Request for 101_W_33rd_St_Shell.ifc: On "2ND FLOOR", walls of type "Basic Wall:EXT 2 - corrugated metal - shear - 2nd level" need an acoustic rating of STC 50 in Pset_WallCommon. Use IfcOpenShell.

First a look at what the model holds.

```python
import ifcopenshell
import ifcopenshell.util.element

model = ifcopenshell.open("101_W_33rd_St_Shell.ifc")
print(model.schema)
storey = next(s for s in model.by_type("IfcBuildingStorey") if s.Name == "2ND FLOOR")
walls = [e for e in ifcopenshell.util.element.get_decomposition(storey) if e.is_a("IfcWall")]
seen = {}
for e in walls:
    element_type = ifcopenshell.util.element.get_type(e)
    key = (element_type.Name if element_type != e and element_type else None, ifcopenshell.util.element.get_pset(e, "Pset_WallCommon", "AcousticRating"))
    seen[key] = seen.get(key, 0) + 1
for (name, value), count in sorted(seen.items(), key=str):
    print(count, "x", name, "|", value)
```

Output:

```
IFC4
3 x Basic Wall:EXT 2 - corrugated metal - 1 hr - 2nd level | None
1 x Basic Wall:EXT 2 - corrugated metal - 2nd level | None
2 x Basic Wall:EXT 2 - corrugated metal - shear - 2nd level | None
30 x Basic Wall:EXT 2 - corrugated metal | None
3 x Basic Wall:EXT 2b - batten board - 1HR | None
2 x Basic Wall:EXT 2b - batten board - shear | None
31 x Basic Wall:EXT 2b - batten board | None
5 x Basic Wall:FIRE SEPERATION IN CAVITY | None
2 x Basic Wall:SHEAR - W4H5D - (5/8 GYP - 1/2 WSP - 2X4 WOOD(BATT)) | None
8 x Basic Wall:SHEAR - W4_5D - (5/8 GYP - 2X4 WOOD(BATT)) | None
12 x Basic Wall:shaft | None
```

```python
import ifcopenshell
import ifcopenshell.api.pset
import ifcopenshell.util.element

model = ifcopenshell.open("101_W_33rd_St_Shell.ifc")

storey = next(s for s in model.by_type("IfcBuildingStorey") if s.Name == "2ND FLOOR")
walls = [e for e in ifcopenshell.util.element.get_decomposition(storey) if e.is_a("IfcWall")]

count = 0
for e in walls:
    element_type = ifcopenshell.util.element.get_type(e)
    if element_type in (None, e) or element_type.Name != "Basic Wall:EXT 2 - corrugated metal - shear - 2nd level":
        continue
    # add_pset returns the element's existing set when there is one.
    pset = ifcopenshell.api.pset.add_pset(model, product=e, name="Pset_WallCommon")
    ifcopenshell.api.pset.edit_pset(model, pset=pset, properties={"AcousticRating": "STC 50"})
    count += 1

print(count, "walls updated")

model.write("101_W_33rd_St_Shell_rev.ifc")
```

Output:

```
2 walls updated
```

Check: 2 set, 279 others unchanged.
